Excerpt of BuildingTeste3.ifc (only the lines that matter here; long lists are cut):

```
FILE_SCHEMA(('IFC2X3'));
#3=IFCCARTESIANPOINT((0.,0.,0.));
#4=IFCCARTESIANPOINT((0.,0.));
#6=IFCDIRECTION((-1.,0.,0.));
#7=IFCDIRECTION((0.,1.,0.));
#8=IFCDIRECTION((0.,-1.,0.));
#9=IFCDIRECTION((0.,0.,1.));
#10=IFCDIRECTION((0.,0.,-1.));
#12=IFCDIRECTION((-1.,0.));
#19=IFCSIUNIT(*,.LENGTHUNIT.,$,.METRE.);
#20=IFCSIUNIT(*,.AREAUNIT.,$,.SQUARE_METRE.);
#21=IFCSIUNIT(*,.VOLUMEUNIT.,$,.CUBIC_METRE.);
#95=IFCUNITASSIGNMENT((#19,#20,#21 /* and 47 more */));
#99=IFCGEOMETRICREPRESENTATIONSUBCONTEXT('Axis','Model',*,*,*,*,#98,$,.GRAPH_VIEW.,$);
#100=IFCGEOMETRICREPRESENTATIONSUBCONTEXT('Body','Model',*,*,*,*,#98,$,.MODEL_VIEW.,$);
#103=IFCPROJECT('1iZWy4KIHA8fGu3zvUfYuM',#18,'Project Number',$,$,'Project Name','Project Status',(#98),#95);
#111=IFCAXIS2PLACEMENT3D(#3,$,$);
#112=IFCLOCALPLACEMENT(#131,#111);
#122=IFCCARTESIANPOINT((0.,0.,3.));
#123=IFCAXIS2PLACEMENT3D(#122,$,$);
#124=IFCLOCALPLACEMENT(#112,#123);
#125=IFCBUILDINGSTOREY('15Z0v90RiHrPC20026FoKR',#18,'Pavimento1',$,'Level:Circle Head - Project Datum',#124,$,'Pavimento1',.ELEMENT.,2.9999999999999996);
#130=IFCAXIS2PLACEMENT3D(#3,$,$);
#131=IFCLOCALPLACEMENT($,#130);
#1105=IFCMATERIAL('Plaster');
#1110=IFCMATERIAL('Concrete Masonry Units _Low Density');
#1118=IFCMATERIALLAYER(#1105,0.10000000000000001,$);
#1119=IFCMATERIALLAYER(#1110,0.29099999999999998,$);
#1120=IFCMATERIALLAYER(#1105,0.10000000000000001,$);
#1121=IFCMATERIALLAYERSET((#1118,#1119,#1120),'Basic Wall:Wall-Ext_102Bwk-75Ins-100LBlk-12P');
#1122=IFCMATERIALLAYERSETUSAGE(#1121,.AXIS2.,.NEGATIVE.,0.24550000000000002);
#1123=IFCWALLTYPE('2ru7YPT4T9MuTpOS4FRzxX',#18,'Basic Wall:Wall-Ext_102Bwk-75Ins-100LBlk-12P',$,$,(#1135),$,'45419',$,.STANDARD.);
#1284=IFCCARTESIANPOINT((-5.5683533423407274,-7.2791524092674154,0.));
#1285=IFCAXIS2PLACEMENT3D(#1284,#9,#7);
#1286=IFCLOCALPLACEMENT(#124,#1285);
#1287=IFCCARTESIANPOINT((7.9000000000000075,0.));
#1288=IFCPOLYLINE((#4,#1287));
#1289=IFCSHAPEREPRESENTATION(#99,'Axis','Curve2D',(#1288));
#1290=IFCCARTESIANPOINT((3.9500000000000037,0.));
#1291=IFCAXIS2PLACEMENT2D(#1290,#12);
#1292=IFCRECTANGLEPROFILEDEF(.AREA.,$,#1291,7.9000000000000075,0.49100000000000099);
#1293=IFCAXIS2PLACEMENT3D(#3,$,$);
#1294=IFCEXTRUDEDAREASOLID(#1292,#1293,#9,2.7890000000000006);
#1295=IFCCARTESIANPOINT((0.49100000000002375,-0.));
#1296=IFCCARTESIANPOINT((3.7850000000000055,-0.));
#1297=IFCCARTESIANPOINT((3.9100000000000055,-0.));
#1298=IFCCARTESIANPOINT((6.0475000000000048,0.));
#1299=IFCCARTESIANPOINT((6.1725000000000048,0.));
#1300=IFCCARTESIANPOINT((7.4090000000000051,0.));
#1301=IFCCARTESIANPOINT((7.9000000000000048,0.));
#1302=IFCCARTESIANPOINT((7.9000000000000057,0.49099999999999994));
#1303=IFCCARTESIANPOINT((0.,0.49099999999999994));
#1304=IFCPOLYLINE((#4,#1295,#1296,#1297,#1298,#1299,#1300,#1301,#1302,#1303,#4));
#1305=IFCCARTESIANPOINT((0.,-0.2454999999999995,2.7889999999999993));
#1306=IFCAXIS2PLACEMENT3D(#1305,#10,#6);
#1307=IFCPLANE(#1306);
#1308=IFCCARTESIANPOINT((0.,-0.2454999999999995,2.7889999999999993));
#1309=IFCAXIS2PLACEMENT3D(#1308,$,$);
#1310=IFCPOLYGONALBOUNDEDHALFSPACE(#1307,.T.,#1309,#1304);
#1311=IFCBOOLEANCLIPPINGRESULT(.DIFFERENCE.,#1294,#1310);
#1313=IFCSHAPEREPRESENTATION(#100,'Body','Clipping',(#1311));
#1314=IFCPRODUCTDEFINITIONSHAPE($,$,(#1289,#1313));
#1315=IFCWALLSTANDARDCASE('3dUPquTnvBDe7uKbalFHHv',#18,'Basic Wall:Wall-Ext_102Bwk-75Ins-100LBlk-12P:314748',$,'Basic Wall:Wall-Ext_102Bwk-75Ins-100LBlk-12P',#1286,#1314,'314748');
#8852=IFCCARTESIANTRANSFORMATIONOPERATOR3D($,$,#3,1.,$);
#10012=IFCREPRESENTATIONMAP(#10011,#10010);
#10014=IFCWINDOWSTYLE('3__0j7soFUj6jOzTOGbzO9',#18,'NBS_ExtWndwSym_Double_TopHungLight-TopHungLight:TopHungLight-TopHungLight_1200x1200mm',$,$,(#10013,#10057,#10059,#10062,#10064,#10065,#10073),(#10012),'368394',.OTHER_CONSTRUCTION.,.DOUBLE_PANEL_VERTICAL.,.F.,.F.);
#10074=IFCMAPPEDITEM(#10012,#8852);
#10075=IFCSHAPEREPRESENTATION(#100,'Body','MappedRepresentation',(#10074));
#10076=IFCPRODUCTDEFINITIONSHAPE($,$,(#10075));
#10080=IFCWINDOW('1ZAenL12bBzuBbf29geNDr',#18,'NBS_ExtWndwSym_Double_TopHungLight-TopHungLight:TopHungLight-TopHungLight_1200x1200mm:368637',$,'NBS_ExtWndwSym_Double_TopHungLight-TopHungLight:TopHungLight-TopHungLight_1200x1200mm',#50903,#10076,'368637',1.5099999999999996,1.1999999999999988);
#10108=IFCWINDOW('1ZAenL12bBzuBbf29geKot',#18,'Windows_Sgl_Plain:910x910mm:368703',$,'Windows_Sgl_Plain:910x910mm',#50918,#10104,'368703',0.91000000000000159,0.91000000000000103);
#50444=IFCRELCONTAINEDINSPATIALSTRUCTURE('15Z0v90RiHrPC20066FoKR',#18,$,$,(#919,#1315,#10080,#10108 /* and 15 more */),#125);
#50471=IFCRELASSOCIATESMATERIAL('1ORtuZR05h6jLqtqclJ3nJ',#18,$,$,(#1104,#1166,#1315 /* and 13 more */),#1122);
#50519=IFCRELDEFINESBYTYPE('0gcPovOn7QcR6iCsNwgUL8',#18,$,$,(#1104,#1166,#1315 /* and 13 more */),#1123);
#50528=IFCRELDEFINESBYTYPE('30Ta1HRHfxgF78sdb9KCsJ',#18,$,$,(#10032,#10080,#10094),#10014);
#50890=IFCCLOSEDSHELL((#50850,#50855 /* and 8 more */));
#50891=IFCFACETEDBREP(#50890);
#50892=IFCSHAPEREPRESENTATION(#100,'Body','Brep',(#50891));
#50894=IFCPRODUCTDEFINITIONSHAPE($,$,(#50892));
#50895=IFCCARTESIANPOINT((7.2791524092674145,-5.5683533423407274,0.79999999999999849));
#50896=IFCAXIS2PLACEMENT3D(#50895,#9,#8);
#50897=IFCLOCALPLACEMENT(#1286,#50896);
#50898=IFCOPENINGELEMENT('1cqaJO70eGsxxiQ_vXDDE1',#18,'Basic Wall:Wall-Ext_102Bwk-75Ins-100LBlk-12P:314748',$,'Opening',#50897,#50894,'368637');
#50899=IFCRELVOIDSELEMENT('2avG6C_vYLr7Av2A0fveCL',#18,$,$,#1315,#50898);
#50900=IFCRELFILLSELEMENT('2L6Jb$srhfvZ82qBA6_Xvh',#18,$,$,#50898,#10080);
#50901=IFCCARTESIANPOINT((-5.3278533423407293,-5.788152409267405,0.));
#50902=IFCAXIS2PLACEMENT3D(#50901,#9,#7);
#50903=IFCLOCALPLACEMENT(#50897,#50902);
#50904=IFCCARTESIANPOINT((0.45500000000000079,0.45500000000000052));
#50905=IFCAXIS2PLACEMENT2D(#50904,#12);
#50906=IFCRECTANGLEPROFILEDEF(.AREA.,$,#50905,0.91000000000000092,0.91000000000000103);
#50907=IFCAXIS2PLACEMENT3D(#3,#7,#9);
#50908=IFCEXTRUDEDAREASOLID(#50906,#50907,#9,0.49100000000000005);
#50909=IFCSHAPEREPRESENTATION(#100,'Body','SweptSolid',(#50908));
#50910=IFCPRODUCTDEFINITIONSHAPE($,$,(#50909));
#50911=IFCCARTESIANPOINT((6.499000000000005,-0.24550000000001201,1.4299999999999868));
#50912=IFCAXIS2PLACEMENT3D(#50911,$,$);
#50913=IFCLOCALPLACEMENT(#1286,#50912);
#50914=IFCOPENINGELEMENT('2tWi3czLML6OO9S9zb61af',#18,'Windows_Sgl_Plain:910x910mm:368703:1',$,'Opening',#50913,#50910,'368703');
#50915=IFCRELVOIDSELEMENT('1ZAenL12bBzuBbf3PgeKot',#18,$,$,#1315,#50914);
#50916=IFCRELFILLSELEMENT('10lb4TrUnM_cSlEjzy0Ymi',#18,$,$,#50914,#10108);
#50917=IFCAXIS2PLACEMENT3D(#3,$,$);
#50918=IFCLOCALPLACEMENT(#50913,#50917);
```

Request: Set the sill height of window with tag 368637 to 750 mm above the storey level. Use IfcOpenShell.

```python
import numpy as np
import ifcopenshell
import ifcopenshell.api.geometry
import ifcopenshell.geom
import ifcopenshell.util.element
import ifcopenshell.util.placement
import ifcopenshell.util.shape
import ifcopenshell.util.unit

model = ifcopenshell.open("BuildingTeste3.ifc")
unit_scale = ifcopenshell.util.unit.calculate_unit_scale(model)

window = model.by_guid("1ZAenL12bBzuBbf29geNDr")
opening = window.FillsVoids[0].RelatingOpeningElement
storey = ifcopenshell.util.element.get_container(window, ifc_class="IfcBuildingStorey")
level = ifcopenshell.util.placement.get_local_placement(storey.ObjectPlacement)[2, 3]

# The opening's origin need not be at the sill, so measure its lowest point.
shape = ifcopenshell.geom.create_shape(ifcopenshell.geom.settings(), opening)
bottom = ifcopenshell.util.shape.get_shape_bottom_elevation(shape, shape.geometry) / unit_scale
dz = level + 0.75 / unit_scale - bottom

shift = np.array([0.0, 0.0, dz])
# The window is placed relative to its opening, so it follows when the opening moves.
matrix = ifcopenshell.util.placement.get_local_placement(opening.ObjectPlacement)
matrix[:3, 3] += shift
ifcopenshell.api.geometry.edit_object_placement(
    model, product=opening, matrix=matrix, is_si=False, should_transform_children=True
)

print(f"moved by {dz * unit_scale:+.3f} m")

model.write("BuildingTeste3_v2.ifc")
```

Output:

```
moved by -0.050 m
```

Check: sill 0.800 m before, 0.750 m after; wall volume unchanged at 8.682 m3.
